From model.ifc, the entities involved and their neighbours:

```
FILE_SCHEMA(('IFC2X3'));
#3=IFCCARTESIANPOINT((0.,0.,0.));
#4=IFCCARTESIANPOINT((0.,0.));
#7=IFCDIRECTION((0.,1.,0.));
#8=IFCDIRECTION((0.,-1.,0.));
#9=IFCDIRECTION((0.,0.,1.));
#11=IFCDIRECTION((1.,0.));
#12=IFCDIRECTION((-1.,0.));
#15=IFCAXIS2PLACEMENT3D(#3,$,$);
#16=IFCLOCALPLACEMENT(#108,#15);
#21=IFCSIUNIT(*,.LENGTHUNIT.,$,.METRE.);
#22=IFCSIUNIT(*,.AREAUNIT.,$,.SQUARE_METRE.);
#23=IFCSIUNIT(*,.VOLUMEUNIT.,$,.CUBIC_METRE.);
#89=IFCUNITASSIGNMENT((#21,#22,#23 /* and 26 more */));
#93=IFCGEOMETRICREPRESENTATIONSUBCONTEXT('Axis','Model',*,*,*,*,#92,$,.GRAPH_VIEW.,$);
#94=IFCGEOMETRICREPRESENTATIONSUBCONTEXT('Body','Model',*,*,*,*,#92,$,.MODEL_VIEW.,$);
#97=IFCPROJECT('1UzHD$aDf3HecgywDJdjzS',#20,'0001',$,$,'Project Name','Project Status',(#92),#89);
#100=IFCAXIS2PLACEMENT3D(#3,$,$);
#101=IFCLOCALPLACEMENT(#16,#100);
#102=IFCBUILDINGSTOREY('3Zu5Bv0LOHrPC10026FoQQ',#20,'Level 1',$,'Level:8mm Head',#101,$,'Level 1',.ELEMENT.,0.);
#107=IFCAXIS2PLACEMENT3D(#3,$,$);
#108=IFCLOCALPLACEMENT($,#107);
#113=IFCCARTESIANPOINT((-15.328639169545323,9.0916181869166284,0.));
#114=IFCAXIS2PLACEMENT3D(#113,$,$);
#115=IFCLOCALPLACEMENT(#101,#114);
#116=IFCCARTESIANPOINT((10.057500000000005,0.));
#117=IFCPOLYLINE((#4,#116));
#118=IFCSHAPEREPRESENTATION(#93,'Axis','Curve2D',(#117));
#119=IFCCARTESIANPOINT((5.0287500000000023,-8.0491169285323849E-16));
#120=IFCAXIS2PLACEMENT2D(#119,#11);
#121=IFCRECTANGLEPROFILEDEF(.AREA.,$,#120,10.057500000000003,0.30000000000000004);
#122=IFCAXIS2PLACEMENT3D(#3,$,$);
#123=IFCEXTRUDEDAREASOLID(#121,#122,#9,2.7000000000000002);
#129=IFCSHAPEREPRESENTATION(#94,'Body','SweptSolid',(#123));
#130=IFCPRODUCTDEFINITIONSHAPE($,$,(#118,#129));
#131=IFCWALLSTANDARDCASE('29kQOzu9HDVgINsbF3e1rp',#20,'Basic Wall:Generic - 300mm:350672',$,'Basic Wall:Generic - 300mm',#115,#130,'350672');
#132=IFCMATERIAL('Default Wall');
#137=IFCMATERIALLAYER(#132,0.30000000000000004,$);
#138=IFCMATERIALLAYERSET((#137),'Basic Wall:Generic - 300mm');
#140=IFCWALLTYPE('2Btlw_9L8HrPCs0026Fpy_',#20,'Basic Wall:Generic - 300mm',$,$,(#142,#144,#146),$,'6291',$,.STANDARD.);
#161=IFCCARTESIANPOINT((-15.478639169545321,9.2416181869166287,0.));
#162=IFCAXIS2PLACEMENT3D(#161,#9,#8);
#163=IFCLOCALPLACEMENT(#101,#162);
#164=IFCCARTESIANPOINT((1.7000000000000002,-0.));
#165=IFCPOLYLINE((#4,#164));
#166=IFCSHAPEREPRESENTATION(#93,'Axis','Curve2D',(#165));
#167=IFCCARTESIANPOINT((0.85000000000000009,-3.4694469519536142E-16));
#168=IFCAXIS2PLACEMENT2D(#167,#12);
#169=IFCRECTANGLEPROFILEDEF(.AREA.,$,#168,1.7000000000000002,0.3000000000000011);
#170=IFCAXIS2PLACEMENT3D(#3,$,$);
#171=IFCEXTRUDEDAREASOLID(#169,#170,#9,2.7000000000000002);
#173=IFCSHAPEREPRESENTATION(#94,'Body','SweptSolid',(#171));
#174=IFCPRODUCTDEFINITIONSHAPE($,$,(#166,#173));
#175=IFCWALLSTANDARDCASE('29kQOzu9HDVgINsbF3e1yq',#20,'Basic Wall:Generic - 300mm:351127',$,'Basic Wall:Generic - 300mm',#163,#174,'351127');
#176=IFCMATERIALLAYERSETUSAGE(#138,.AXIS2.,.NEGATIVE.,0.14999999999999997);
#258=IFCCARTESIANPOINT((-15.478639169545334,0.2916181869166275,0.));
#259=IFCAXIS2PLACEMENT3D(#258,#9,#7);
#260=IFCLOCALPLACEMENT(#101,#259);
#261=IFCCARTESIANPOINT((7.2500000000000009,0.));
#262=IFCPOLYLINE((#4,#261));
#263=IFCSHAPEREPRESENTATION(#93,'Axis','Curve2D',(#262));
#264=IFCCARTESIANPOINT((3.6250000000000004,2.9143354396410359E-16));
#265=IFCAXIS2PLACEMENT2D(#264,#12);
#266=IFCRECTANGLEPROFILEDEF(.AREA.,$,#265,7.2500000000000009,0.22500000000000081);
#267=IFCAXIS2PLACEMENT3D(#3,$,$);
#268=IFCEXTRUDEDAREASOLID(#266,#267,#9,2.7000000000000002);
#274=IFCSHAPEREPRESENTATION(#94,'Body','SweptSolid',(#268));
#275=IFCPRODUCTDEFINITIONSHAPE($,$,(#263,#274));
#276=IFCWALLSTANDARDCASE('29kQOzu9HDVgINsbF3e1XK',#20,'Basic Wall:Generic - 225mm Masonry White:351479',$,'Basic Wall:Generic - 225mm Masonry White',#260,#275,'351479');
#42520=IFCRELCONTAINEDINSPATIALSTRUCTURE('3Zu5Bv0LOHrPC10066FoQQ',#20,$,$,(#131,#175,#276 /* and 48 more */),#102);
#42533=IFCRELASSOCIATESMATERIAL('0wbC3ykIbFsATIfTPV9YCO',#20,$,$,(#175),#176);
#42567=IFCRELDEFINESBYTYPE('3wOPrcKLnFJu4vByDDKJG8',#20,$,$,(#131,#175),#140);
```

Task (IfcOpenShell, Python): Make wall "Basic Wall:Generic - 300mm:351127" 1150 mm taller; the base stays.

```python
import ifcopenshell
import ifcopenshell.geom
import ifcopenshell.util.representation
import ifcopenshell.util.shape
import ifcopenshell.util.unit

model = ifcopenshell.open("model.ifc")
unit_scale = ifcopenshell.util.unit.calculate_unit_scale(model)
settings = ifcopenshell.geom.settings()


def volume(element):
    """Net volume in cubic metres, openings subtracted."""
    shape = ifcopenshell.geom.create_shape(settings, element)
    return ifcopenshell.util.shape.get_volume(shape.geometry)


wall = model.by_guid("29kQOzu9HDVgINsbF3e1yq")
before = volume(wall)

body = ifcopenshell.util.representation.get_representation(wall, "Model", "Body")
solid = body.Items[0]
old_height = solid.Depth
solid.Depth += 1.15 / unit_scale
after = volume(wall)

print(f"height {old_height:g} -> {solid.Depth:g}, volume {before:.3f} -> {after:.3f} m3")

model.write("model_rev.ifc")
```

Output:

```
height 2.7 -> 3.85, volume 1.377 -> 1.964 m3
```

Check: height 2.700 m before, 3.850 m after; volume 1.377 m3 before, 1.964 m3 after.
